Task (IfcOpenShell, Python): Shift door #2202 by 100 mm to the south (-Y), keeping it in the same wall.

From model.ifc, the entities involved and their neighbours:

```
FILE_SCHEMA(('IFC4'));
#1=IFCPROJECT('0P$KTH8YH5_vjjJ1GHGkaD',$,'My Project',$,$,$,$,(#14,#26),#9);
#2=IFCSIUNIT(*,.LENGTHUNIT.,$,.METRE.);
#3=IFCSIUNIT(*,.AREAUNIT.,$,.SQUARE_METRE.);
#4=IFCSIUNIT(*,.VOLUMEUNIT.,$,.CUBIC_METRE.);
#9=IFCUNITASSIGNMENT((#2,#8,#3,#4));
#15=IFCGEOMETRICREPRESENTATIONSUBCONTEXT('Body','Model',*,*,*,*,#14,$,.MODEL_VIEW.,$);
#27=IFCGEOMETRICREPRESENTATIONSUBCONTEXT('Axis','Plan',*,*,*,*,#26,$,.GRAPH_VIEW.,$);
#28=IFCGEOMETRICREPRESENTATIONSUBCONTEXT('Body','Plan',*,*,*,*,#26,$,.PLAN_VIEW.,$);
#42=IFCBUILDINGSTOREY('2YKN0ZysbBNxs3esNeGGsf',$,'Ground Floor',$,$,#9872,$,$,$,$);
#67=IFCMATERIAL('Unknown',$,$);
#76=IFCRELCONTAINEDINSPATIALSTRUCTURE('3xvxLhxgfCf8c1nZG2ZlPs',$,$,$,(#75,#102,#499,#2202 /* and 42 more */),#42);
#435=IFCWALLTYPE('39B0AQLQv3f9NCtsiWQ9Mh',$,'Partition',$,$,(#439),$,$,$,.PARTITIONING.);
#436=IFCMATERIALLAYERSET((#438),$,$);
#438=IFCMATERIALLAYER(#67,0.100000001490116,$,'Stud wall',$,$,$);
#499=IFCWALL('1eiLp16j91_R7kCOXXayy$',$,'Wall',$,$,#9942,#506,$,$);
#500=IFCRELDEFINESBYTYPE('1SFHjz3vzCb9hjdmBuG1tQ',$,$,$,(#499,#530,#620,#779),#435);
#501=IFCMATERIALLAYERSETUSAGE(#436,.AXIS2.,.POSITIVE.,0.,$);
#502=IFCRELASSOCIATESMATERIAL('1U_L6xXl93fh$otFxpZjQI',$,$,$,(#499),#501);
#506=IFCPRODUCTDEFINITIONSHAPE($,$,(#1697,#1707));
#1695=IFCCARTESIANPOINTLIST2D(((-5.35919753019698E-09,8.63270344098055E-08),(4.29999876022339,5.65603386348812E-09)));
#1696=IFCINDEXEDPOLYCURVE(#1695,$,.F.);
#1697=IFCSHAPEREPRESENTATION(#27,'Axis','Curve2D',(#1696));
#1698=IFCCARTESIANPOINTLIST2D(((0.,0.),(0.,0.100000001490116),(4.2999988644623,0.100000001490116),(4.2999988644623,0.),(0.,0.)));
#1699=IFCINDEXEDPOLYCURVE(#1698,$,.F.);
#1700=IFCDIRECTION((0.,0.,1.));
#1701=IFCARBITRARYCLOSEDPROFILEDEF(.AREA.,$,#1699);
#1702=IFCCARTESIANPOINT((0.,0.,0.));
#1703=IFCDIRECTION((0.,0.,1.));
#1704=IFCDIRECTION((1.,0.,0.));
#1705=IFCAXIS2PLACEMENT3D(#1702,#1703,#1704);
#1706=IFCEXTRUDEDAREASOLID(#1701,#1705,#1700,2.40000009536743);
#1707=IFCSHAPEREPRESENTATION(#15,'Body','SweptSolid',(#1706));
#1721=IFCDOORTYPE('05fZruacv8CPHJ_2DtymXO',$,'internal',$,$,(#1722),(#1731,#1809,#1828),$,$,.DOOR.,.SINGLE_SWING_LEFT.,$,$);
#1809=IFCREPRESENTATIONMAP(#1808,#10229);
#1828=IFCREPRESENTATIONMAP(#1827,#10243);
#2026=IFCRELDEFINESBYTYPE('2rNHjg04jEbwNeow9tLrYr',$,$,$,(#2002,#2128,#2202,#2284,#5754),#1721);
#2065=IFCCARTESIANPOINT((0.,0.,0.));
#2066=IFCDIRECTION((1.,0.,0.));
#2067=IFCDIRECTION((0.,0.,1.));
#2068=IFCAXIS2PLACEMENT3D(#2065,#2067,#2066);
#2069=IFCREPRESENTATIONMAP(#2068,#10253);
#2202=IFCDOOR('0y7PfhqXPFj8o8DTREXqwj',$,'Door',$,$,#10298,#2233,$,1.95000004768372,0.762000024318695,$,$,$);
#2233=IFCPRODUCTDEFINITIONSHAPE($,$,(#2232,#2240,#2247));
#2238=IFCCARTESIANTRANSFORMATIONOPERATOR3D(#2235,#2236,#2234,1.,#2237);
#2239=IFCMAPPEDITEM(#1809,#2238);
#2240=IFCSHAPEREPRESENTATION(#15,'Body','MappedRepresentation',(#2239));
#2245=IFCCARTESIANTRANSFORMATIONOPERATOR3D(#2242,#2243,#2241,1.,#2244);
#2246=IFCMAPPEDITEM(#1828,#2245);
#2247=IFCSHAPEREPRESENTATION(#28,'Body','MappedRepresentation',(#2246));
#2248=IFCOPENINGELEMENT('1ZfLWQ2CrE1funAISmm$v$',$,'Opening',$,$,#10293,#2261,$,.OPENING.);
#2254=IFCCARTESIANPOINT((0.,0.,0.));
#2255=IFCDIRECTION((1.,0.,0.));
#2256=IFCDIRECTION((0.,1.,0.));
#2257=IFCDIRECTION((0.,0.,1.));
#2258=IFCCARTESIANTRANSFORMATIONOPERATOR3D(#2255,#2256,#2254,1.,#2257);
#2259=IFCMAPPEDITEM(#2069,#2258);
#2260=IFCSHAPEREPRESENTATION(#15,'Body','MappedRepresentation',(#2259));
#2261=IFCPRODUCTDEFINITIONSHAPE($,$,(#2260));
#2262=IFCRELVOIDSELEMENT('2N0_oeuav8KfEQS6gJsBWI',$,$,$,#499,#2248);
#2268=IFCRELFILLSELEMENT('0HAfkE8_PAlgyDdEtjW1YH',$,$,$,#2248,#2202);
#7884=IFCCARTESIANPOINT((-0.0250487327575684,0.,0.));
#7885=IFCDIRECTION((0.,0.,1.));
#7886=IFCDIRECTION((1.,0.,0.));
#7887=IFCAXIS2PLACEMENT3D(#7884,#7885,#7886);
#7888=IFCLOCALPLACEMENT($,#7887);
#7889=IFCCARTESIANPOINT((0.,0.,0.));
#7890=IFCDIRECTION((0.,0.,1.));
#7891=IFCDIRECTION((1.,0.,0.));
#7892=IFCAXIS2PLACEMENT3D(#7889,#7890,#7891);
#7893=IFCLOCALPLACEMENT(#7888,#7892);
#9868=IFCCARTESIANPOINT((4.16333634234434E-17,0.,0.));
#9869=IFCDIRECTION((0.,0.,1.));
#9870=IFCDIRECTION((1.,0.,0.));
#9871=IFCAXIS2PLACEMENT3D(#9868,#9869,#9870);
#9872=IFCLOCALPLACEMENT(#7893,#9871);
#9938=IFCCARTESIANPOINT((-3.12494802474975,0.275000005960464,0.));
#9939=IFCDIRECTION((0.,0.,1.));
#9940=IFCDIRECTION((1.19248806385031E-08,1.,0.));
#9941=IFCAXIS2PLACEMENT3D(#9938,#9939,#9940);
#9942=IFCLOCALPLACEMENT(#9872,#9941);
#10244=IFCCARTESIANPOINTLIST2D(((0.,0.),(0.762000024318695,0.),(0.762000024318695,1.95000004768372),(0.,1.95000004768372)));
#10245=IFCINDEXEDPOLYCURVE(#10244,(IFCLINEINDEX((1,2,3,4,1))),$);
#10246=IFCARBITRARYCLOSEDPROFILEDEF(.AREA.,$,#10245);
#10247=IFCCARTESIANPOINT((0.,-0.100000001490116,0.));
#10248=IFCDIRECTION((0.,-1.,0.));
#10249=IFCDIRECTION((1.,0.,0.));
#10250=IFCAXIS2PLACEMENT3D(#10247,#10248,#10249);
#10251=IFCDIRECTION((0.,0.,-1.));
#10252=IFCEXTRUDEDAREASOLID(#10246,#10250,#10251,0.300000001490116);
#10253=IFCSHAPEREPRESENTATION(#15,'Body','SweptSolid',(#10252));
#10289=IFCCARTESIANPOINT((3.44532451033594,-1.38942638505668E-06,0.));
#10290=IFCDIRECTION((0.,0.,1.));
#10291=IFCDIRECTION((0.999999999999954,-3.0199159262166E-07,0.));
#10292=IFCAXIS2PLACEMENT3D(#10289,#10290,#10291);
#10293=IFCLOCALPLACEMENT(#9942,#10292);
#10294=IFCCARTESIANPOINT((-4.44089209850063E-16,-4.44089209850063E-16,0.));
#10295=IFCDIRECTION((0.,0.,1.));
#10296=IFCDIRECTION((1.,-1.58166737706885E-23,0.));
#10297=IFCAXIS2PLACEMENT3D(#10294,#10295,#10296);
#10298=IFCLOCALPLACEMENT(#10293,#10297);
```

```python
import ifcopenshell
import ifcopenshell.api.geometry
import ifcopenshell.util.placement

model = ifcopenshell.open("model.ifc")

door = model.by_id(2202)
opening = door.FillsVoids[0].RelatingOpeningElement
wall = opening.VoidsElements[0].RelatingBuildingElement

wall_matrix = ifcopenshell.util.placement.get_local_placement(wall.ObjectPlacement)
shift = wall_matrix[:3, 0] * -0.1
before = ifcopenshell.util.placement.get_local_placement(door.ObjectPlacement)[:3, 3].copy()

# The door is placed relative to its opening, so it follows when the opening moves.
matrix = ifcopenshell.util.placement.get_local_placement(opening.ObjectPlacement)
matrix[:3, 3] += shift
ifcopenshell.api.geometry.edit_object_placement(
    model, product=opening, matrix=matrix, is_si=False, should_transform_children=True
)

after = ifcopenshell.util.placement.get_local_placement(door.ObjectPlacement)[:3, 3]
print("door moved by", (after - before).round(3) + 0.0)

model.write("model_rev.ifc")
```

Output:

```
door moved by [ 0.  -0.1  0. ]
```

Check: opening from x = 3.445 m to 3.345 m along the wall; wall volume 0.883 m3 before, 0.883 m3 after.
